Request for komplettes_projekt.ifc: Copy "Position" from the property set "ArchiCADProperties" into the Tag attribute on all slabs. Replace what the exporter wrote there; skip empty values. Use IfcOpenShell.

First a look at what the model holds.

```python
import ifcopenshell
import ifcopenshell.util.element

model = ifcopenshell.open("komplettes_projekt.ifc")
print(model.schema)
slabs = model.by_type("IfcSlab")
print(len(slabs), "slabs")
for e in slabs[:8]:
    source = ifcopenshell.util.element.get_pset(e, "ArchiCADProperties", "Position")
    target = e.Tag
    print(e.id(), repr(source), repr(target), sep=" | ")
```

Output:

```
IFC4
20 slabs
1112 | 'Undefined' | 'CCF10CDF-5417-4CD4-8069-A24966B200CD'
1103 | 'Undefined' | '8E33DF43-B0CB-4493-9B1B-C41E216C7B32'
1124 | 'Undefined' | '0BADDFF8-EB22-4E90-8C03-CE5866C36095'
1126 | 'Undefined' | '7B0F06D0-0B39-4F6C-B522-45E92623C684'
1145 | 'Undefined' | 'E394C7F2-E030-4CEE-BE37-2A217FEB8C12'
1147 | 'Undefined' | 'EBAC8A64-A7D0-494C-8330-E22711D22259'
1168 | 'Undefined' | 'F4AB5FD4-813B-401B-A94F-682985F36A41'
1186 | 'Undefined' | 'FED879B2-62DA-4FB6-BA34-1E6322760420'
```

```python
import ifcopenshell
import ifcopenshell.util.element

model = ifcopenshell.open("komplettes_projekt.ifc")

count = 0
for e in model.by_type("IfcSlab"):
    value = ifcopenshell.util.element.get_pset(e, "ArchiCADProperties", "Position")
    current = e.Tag
    if not value or not value.strip() or current == value:
        continue
    e.Tag = value
    count += 1

print(count, "slabs updated")

model.write("komplettes_projekt_v2.ifc")
```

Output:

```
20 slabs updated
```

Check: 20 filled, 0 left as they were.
